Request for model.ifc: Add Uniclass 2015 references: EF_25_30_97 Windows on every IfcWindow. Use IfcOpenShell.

First a look at what the model holds.

```python
import ifcopenshell

model = ifcopenshell.open("model.ifc")
print(model.schema)
print("classifications:", [c.Name for c in model.by_type("IfcClassification")])
for ifc_class in ("IfcDoor", "IfcRoof", "IfcStair", "IfcWall", "IfcWindow"):
    print(ifc_class, len(model.by_type(ifc_class)))
```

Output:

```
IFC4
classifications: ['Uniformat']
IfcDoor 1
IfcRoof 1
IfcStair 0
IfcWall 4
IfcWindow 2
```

```python
import ifcopenshell
import ifcopenshell.api.classification

model = ifcopenshell.open("model.ifc")

system = ifcopenshell.api.classification.add_classification(model, classification="Uniclass 2015")

codes = {
    "IfcWindow": ("EF_25_30_97", "Windows"),
}
for ifc_class, (code, name) in codes.items():
    products = model.by_type(ifc_class)
    ifcopenshell.api.classification.add_reference(
        model, products=products, classification=system, identification=code, name=name
    )
    print(code, len(products))

model.write("model-out.ifc")
```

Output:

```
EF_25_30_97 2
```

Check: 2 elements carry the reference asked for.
